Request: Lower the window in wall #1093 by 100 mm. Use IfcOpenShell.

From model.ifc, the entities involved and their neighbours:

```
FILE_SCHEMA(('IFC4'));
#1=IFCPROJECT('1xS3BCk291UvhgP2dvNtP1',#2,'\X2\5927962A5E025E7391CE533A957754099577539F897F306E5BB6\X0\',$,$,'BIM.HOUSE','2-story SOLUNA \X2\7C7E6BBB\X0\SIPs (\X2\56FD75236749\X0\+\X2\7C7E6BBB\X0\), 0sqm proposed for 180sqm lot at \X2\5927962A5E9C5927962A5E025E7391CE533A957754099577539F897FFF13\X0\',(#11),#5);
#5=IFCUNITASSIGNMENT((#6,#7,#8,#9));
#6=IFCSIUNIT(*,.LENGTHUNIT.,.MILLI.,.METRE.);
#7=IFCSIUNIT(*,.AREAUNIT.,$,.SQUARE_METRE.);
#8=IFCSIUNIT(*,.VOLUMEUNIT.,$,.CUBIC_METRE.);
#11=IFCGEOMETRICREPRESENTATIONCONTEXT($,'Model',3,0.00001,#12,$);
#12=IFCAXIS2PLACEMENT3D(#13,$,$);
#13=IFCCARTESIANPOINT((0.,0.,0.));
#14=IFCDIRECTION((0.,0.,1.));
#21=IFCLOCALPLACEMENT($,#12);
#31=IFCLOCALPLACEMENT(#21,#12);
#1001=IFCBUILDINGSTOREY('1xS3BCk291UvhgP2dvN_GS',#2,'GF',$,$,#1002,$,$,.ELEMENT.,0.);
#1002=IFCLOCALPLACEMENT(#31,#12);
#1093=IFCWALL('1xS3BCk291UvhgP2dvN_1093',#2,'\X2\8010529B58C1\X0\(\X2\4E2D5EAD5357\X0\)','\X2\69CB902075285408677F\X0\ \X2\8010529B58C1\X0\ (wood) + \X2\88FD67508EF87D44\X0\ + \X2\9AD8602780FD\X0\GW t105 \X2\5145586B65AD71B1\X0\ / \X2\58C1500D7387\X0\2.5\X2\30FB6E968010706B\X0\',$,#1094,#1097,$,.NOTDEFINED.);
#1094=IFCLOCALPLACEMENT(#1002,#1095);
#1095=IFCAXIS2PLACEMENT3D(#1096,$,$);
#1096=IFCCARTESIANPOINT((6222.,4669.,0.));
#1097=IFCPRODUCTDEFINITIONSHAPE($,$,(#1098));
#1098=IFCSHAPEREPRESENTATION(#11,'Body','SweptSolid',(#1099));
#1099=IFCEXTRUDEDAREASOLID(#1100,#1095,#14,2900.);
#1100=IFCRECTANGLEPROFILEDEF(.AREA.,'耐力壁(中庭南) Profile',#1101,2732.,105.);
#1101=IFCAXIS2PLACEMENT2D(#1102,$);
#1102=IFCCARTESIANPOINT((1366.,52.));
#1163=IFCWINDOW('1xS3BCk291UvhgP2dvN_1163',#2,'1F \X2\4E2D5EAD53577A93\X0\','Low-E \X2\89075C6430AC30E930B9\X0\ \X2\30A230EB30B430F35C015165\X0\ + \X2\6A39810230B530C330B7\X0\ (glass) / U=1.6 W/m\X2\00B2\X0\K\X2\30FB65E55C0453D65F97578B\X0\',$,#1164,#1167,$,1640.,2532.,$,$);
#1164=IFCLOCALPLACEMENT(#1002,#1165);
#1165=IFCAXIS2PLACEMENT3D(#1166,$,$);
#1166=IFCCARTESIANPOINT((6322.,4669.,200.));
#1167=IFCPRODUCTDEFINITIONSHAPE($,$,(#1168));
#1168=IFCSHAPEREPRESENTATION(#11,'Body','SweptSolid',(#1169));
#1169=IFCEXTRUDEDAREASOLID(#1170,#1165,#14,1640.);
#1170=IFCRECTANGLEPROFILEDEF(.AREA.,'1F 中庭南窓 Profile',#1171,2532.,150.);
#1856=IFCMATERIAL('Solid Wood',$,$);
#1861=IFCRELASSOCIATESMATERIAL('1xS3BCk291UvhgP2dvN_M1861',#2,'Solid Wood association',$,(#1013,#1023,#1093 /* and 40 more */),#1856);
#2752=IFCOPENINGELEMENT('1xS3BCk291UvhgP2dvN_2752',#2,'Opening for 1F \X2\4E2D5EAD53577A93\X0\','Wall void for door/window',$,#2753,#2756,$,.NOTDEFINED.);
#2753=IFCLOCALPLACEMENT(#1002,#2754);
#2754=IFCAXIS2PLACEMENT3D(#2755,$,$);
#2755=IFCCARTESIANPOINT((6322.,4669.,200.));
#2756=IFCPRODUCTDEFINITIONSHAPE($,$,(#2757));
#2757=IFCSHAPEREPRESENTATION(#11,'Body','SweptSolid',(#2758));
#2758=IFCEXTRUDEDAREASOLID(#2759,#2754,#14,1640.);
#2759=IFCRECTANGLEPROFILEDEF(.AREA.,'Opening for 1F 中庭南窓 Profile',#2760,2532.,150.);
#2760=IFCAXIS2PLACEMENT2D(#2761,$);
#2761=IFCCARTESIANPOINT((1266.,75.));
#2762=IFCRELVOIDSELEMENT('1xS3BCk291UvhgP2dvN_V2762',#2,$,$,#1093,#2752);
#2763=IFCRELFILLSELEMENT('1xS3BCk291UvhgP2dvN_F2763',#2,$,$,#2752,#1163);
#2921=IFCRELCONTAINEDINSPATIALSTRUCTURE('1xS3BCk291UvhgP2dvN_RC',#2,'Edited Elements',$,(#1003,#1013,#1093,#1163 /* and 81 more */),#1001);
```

```python
import numpy as np
import ifcopenshell
import ifcopenshell.api.geometry
import ifcopenshell.util.placement
import ifcopenshell.util.unit

model = ifcopenshell.open("model.ifc")
unit_scale = ifcopenshell.util.unit.calculate_unit_scale(model)

window = model.by_guid("1xS3BCk291UvhgP2dvN_1163")
opening = window.FillsVoids[0].RelatingOpeningElement
dz = -0.1 / unit_scale

shift = np.array([0.0, 0.0, dz])
# The window is not placed relative to its opening, so move both.
for product in (opening, window):
    matrix = ifcopenshell.util.placement.get_local_placement(product.ObjectPlacement)
    matrix[:3, 3] += shift
    ifcopenshell.api.geometry.edit_object_placement(model, product=product, matrix=matrix, is_si=False)

print(f"moved by {dz * unit_scale:+.3f} m")

model.write("model-out.ifc")
```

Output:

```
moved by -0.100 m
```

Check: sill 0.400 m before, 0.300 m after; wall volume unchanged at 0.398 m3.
